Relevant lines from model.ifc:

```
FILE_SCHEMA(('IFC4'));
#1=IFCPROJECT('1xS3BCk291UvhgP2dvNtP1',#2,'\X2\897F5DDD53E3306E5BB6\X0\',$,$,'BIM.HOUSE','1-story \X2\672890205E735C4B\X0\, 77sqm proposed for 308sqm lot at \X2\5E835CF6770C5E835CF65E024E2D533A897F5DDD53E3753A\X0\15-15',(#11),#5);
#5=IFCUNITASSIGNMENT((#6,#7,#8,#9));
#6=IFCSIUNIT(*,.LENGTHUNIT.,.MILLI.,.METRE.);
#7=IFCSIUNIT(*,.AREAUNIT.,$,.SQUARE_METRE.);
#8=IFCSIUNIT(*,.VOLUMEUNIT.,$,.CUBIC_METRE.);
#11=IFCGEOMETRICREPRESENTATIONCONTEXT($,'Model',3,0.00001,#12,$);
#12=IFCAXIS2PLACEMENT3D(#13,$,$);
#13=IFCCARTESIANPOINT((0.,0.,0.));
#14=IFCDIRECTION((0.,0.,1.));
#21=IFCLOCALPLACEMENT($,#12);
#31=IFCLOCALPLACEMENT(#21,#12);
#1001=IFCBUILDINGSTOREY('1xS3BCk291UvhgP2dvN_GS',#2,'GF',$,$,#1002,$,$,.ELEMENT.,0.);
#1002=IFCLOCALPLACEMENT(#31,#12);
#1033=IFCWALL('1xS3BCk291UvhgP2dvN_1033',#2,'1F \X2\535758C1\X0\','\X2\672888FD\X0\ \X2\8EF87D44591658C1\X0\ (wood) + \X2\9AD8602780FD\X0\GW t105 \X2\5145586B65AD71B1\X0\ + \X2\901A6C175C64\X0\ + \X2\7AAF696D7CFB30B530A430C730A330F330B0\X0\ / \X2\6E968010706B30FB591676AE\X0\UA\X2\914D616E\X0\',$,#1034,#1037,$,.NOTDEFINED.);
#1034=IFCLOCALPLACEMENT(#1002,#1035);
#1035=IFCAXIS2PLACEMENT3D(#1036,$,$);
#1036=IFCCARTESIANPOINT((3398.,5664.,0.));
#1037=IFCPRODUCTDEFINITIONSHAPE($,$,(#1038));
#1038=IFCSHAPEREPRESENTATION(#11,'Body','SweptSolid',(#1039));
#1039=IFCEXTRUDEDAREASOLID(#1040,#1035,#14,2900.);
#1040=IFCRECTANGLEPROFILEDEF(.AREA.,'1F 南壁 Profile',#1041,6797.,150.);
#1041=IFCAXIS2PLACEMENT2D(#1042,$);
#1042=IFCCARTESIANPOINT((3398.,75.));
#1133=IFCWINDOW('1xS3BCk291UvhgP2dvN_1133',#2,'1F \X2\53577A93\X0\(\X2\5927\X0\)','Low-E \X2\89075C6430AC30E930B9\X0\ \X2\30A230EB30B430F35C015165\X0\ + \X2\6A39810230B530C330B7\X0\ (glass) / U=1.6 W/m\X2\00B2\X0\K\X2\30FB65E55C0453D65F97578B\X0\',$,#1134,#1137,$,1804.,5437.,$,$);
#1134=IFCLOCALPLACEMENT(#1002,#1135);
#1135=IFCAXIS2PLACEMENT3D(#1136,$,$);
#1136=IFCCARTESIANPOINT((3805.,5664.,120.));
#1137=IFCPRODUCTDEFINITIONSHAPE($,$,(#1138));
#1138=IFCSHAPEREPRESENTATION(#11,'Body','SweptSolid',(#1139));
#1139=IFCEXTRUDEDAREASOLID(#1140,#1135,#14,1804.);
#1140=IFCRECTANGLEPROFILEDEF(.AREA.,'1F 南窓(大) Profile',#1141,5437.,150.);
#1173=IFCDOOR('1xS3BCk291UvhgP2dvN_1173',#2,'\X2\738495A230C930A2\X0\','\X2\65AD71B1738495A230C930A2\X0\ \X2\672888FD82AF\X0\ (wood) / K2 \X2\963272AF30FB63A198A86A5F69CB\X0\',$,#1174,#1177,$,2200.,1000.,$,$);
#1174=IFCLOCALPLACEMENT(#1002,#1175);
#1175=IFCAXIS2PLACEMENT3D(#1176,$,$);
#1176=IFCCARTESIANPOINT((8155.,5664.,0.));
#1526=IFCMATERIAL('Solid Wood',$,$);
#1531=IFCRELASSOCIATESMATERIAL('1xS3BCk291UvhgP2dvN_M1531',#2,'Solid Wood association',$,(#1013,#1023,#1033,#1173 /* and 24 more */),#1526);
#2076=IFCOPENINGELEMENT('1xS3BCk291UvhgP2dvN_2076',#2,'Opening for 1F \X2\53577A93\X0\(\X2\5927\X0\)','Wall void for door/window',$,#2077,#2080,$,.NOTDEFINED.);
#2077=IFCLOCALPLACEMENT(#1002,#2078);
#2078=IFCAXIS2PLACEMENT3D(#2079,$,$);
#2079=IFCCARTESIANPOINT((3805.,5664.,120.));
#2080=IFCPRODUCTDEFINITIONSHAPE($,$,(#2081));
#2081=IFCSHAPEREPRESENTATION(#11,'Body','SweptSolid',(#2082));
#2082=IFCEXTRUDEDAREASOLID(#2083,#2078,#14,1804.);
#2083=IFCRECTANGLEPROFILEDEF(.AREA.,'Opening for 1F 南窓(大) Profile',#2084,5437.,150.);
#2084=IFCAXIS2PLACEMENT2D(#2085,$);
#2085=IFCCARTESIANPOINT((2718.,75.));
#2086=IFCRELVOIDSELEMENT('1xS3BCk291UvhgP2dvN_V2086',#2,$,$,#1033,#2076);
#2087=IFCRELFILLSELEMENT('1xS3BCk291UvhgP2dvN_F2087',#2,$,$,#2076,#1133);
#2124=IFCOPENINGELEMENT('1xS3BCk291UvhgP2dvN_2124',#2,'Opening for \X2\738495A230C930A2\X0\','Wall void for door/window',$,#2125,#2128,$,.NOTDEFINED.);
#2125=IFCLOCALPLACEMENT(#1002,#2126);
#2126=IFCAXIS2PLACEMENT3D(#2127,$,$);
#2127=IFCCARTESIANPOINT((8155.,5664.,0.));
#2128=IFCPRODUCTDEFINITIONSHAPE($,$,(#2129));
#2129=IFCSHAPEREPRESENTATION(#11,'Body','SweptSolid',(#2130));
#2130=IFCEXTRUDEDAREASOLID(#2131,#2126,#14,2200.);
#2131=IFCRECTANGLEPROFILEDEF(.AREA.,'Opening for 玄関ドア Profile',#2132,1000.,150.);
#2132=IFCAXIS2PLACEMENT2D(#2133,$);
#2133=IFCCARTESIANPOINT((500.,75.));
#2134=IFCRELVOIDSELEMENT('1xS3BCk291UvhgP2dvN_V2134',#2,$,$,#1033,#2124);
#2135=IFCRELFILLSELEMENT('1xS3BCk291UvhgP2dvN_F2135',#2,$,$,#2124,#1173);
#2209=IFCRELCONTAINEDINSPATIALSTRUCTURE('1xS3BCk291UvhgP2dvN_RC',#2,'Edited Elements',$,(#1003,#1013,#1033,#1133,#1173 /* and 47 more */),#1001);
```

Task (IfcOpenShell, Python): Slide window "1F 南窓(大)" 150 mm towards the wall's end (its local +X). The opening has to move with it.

```python
import ifcopenshell
import ifcopenshell.api.geometry
import ifcopenshell.util.placement
import ifcopenshell.util.unit

model = ifcopenshell.open("model.ifc")
unit_scale = ifcopenshell.util.unit.calculate_unit_scale(model)

window = model.by_guid("1xS3BCk291UvhgP2dvN_1133")
opening = window.FillsVoids[0].RelatingOpeningElement
wall = opening.VoidsElements[0].RelatingBuildingElement

wall_matrix = ifcopenshell.util.placement.get_local_placement(wall.ObjectPlacement)
shift = wall_matrix[:3, 0] * 0.15 / unit_scale
before = ifcopenshell.util.placement.get_local_placement(window.ObjectPlacement)[:3, 3].copy()

# The window is not placed relative to its opening, so move both.
for product in (opening, window):
    matrix = ifcopenshell.util.placement.get_local_placement(product.ObjectPlacement)
    matrix[:3, 3] += shift
    ifcopenshell.api.geometry.edit_object_placement(model, product=product, matrix=matrix, is_si=False)

after = ifcopenshell.util.placement.get_local_placement(window.ObjectPlacement)[:3, 3]
print("window moved by", (after - before).round(3) + 0.0)

model.write("model_updated.ifc")
```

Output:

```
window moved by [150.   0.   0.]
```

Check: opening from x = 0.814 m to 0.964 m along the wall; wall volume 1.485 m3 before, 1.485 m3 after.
